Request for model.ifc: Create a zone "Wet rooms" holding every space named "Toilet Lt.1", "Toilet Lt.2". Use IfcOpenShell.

First a look at what the model holds.

```python
import ifcopenshell

model = ifcopenshell.open("model.ifc")
print(model.schema)
seen = {}
for space in model.by_type("IfcSpace"):
    seen[space.Name] = seen.get(space.Name, 0) + 1
for name, count in sorted(seen.items(), key=str):
    print(count, "x", name)
print("zones:", [z.Name for z in model.by_type("IfcZone")][:20])
```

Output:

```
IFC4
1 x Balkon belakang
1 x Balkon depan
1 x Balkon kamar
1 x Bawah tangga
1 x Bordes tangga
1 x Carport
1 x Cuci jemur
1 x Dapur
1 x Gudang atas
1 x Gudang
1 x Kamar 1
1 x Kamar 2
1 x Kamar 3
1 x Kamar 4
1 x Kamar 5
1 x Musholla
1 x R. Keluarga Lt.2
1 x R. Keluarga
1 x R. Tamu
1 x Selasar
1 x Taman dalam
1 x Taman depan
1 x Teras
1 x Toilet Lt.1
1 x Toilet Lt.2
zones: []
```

```python
import ifcopenshell
import ifcopenshell.api.group
import ifcopenshell.api.root

model = ifcopenshell.open("model.ifc")

names = {"Toilet Lt.1", "Toilet Lt.2"}
spaces = [s for s in model.by_type("IfcSpace") if s.Name in names]

zone = ifcopenshell.api.root.create_entity(model, ifc_class="IfcZone", name="Wet rooms")
ifcopenshell.api.group.assign_group(model, products=spaces, group=zone)
print(len(spaces), "spaces in", zone.Name)

model.write("model_rev.ifc")
```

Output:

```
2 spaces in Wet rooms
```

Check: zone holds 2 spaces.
